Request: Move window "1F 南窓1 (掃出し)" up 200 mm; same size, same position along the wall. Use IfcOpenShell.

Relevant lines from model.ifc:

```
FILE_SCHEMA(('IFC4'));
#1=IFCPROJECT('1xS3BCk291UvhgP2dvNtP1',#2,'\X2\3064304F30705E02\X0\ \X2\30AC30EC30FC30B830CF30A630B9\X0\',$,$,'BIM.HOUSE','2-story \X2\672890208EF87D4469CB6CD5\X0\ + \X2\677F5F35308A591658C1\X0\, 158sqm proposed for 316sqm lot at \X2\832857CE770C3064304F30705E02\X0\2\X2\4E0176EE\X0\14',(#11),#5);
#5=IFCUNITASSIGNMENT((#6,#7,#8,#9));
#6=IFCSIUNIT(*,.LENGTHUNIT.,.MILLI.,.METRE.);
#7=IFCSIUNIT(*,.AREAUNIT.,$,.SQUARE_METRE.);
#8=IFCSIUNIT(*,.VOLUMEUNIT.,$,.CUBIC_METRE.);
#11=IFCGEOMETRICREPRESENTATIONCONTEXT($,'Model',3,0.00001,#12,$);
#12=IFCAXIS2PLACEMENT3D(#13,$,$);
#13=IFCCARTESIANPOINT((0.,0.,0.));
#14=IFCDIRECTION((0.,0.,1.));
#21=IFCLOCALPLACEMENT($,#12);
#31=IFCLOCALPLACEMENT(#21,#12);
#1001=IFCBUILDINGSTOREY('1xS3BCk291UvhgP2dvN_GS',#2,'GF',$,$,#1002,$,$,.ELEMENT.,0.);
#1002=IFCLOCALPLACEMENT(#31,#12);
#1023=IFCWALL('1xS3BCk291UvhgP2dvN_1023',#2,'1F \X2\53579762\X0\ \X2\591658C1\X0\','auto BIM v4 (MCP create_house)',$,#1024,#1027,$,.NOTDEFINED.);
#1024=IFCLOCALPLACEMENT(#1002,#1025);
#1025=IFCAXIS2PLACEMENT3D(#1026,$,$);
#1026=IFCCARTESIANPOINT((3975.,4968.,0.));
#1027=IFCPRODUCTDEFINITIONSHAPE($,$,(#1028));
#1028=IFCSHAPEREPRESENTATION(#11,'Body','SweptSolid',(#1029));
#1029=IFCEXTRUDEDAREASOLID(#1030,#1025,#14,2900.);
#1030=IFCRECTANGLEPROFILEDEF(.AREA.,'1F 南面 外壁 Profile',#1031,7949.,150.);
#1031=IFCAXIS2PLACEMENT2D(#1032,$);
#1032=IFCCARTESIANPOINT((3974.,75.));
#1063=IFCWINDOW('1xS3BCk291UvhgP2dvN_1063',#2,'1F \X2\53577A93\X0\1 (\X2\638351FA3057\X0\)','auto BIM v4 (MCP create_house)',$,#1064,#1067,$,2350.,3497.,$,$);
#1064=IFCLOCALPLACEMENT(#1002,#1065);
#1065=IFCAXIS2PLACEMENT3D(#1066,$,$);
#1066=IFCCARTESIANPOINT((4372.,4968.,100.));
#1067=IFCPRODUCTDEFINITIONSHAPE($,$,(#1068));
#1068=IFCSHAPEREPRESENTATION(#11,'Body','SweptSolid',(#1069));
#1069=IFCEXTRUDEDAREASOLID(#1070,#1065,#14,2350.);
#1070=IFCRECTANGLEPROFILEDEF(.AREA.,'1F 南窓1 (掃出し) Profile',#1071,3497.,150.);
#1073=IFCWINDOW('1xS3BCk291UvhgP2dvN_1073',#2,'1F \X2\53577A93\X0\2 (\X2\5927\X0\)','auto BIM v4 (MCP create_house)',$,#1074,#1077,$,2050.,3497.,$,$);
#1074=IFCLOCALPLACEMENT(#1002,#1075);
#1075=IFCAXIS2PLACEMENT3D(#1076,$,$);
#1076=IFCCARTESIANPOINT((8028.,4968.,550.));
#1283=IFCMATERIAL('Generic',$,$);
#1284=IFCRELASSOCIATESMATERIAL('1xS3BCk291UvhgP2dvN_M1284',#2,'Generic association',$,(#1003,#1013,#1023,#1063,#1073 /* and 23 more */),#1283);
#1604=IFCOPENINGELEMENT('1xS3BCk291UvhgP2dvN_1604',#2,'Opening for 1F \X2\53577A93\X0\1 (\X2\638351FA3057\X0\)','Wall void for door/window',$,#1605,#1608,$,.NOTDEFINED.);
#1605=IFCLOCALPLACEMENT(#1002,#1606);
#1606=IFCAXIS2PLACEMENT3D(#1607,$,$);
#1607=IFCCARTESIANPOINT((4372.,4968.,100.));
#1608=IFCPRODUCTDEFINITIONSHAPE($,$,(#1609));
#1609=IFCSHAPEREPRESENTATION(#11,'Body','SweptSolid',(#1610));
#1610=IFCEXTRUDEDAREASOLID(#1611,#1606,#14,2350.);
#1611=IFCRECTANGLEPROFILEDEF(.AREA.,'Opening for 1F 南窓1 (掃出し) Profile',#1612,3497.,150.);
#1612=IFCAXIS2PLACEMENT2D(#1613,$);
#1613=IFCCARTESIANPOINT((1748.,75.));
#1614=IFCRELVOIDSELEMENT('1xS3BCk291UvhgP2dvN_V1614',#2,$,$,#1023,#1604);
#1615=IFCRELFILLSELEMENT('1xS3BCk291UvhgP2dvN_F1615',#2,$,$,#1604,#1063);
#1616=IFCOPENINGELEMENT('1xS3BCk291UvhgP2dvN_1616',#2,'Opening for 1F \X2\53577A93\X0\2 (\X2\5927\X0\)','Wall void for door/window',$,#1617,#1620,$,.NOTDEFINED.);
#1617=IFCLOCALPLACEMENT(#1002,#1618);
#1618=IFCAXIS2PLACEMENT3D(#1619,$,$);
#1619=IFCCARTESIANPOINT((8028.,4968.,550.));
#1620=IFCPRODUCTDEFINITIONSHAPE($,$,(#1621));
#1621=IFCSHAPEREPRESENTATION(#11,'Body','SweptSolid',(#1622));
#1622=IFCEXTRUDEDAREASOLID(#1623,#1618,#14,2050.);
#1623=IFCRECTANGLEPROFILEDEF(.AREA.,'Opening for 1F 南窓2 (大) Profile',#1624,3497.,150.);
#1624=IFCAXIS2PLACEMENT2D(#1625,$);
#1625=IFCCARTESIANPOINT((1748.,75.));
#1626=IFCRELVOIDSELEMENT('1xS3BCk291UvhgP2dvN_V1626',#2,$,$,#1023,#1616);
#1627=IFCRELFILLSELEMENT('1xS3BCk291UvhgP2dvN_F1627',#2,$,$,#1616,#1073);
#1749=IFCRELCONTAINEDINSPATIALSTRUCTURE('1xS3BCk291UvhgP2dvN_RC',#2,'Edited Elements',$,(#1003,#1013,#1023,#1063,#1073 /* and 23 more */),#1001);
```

```python
import numpy as np
import ifcopenshell
import ifcopenshell.api.geometry
import ifcopenshell.util.placement
import ifcopenshell.util.unit

model = ifcopenshell.open("model.ifc")
unit_scale = ifcopenshell.util.unit.calculate_unit_scale(model)

window = model.by_guid("1xS3BCk291UvhgP2dvN_1063")
opening = window.FillsVoids[0].RelatingOpeningElement
dz = 200.0

shift = np.array([0.0, 0.0, dz])
# The window is not placed relative to its opening, so move both.
for product in (opening, window):
    matrix = ifcopenshell.util.placement.get_local_placement(product.ObjectPlacement)
    matrix[:3, 3] += shift
    ifcopenshell.api.geometry.edit_object_placement(model, product=product, matrix=matrix, is_si=False)

print(f"moved by {dz * unit_scale:+.3f} m")

model.write("model_updated.ifc")
```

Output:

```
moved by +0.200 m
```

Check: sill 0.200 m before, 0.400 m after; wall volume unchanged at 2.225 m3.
